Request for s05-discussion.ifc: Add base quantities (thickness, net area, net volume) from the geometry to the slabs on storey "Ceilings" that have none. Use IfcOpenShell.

First a look at what the model holds.

```python
import ifcopenshell
import ifcopenshell.util.element
import ifcopenshell.util.unit

model = ifcopenshell.open("s05-discussion.ifc")
print(model.schema)
for unit_type in ("LENGTHUNIT", "AREAUNIT", "VOLUMEUNIT"):
    print(unit_type, ifcopenshell.util.unit.calculate_unit_scale(model, unit_type))
storey = next(s for s in model.by_type("IfcBuildingStorey") if s.Name == "Ceilings")
slabs = [e for e in ifcopenshell.util.element.get_decomposition(storey) if e.is_a("IfcSlab")]
for e in sorted(slabs, key=lambda e: e.id()):
    print(e.id(), e.is_a(), e.Name, list(ifcopenshell.util.element.get_psets(e, qtos_only=True)), sep=" | ")
```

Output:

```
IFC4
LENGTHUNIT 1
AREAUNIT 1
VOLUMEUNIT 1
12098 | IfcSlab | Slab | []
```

```python
import ifcopenshell
import ifcopenshell.api.pset
import ifcopenshell.geom
import ifcopenshell.util.element
import ifcopenshell.util.shape
import ifcopenshell.util.unit

model = ifcopenshell.open("s05-discussion.ifc")
unit_scale = ifcopenshell.util.unit.calculate_unit_scale(model)
area_scale = ifcopenshell.util.unit.calculate_unit_scale(model, "AREAUNIT")
volume_scale = ifcopenshell.util.unit.calculate_unit_scale(model, "VOLUMEUNIT")
settings = ifcopenshell.geom.settings()

storey = next(s for s in model.by_type("IfcBuildingStorey") if s.Name == "Ceilings")
slabs = [e for e in ifcopenshell.util.element.get_decomposition(storey) if e.is_a("IfcSlab")]

for e in sorted(slabs, key=lambda e: e.id()):
    if ifcopenshell.util.element.get_psets(e, qtos_only=True, should_inherit=False):
        continue
    # Geometry comes back in metres, in the element's own axes.
    shape = ifcopenshell.geom.create_shape(settings, e)
    values = {
        "Width": ifcopenshell.util.shape.get_z(shape.geometry) / unit_scale,
        "NetArea": ifcopenshell.util.shape.get_footprint_area(shape.geometry) / area_scale,
        "NetVolume": ifcopenshell.util.shape.get_volume(shape.geometry) / volume_scale,
    }
    qto = ifcopenshell.api.pset.add_qto(model, product=e, name="Qto_SlabBaseQuantities")
    ifcopenshell.api.pset.edit_qto(model, qto=qto, properties=values)
    print(e.id(), {k: round(v, 3) for k, v in values.items()})

model.write("s05-discussion-out.ifc")
```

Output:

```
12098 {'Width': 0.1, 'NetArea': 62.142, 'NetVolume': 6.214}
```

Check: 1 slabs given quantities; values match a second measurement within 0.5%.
